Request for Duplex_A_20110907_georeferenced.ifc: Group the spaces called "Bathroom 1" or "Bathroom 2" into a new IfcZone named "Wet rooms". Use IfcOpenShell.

First a look at what the model holds.

```python
import ifcopenshell

model = ifcopenshell.open("Duplex_A_20110907_georeferenced.ifc")
print(model.schema)
seen = {}
for space in model.by_type("IfcSpace"):
    seen[space.LongName] = seen.get(space.LongName, 0) + 1
for name, count in sorted(seen.items(), key=str):
    print(count, "x", name)
print("zones:", [z.Name for z in model.by_type("IfcZone")][:20])
```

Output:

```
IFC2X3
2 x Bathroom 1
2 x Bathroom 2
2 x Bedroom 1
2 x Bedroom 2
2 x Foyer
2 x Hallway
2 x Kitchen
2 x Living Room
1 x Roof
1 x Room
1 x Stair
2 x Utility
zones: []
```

```python
import ifcopenshell
import ifcopenshell.api.group
import ifcopenshell.api.root

model = ifcopenshell.open("Duplex_A_20110907_georeferenced.ifc")

names = {"Bathroom 1", "Bathroom 2"}
spaces = [s for s in model.by_type("IfcSpace") if s.LongName in names]

zone = ifcopenshell.api.root.create_entity(model, ifc_class="IfcZone", name="Wet rooms")
ifcopenshell.api.group.assign_group(model, products=spaces, group=zone)
print(len(spaces), "spaces in", zone.Name)

model.write("Duplex_A_20110907_georeferenced-out.ifc")
```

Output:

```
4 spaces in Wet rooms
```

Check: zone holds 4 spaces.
